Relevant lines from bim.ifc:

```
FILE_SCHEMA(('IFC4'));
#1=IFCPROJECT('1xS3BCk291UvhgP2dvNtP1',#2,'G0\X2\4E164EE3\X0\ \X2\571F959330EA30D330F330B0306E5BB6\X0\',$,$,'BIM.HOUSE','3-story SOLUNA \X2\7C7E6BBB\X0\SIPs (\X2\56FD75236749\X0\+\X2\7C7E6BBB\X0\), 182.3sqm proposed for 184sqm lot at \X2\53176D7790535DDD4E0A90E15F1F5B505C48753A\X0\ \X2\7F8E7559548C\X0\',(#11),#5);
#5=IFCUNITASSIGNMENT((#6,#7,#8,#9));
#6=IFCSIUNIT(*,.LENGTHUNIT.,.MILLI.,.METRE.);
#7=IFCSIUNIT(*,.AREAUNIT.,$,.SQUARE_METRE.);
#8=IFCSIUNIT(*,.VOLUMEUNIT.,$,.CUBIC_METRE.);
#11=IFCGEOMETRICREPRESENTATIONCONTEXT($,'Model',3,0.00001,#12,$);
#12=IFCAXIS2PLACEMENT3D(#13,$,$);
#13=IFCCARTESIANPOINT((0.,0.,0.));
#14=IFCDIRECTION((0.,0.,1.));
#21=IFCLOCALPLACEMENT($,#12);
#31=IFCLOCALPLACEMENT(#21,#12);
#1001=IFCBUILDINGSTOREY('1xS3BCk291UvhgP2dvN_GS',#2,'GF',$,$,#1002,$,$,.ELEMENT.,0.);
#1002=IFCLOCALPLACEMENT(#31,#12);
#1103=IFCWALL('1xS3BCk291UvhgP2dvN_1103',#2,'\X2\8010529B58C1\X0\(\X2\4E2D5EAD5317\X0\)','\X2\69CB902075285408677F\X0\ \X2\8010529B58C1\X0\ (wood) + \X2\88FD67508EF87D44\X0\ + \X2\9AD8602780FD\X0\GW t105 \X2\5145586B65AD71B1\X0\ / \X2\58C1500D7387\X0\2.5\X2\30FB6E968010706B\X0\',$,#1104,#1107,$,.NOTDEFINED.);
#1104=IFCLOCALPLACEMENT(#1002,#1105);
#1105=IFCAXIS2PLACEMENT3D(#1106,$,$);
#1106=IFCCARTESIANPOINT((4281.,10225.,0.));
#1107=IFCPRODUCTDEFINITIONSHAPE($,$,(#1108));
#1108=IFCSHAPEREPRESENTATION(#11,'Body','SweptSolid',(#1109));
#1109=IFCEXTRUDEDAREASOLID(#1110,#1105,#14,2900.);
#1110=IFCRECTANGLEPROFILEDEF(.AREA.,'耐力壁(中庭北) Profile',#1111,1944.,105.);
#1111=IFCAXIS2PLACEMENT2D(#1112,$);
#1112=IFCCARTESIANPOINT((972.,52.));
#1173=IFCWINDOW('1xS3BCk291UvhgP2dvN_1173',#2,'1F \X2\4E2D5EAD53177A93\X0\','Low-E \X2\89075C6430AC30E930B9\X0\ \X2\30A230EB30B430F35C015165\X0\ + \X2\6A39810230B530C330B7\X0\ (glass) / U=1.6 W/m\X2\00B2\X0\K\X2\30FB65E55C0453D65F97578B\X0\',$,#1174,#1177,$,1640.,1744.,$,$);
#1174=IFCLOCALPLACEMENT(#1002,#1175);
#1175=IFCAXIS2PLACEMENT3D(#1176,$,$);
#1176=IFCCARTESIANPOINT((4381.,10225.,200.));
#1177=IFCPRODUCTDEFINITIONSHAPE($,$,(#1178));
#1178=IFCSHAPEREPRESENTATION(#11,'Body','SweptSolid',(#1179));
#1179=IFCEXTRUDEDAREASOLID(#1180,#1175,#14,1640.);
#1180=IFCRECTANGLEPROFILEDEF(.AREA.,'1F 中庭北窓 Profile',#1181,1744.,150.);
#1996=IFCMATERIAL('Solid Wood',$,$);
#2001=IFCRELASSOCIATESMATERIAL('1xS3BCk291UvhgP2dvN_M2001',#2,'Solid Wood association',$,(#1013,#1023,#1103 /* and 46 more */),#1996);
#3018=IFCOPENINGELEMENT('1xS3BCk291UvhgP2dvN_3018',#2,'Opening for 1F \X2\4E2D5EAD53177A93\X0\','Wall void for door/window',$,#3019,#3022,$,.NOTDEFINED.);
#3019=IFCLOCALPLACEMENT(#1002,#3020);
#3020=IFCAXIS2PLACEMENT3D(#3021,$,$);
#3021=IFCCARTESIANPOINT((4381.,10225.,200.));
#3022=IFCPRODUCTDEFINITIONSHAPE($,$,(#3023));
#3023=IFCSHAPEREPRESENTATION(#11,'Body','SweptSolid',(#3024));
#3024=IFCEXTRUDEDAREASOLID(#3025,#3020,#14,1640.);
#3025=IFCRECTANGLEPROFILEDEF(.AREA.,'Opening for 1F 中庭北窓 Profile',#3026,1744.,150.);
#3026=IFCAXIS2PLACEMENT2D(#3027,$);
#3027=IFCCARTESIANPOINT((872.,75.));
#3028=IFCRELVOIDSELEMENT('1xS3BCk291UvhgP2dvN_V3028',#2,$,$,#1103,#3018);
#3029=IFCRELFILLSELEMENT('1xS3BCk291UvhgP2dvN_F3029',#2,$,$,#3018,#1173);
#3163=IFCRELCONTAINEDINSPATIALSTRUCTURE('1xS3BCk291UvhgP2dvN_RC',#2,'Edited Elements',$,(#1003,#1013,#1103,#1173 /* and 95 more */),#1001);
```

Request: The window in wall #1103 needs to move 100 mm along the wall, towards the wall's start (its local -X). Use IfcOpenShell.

```python
import ifcopenshell
import ifcopenshell.api.geometry
import ifcopenshell.util.placement
import ifcopenshell.util.unit

model = ifcopenshell.open("bim.ifc")
unit_scale = ifcopenshell.util.unit.calculate_unit_scale(model)

window = model.by_guid("1xS3BCk291UvhgP2dvN_1173")
opening = window.FillsVoids[0].RelatingOpeningElement
wall = opening.VoidsElements[0].RelatingBuildingElement

wall_matrix = ifcopenshell.util.placement.get_local_placement(wall.ObjectPlacement)
shift = wall_matrix[:3, 0] * -0.1 / unit_scale
before = ifcopenshell.util.placement.get_local_placement(window.ObjectPlacement)[:3, 3].copy()

# The window is not placed relative to its opening, so move both.
for product in (opening, window):
    matrix = ifcopenshell.util.placement.get_local_placement(product.ObjectPlacement)
    matrix[:3, 3] += shift
    ifcopenshell.api.geometry.edit_object_placement(model, product=product, matrix=matrix, is_si=False)

after = ifcopenshell.util.placement.get_local_placement(window.ObjectPlacement)[:3, 3]
print("window moved by", (after - before).round(3) + 0.0)

model.write("bim_rev.ifc")
```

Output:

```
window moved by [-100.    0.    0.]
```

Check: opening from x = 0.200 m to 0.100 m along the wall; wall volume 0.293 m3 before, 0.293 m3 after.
